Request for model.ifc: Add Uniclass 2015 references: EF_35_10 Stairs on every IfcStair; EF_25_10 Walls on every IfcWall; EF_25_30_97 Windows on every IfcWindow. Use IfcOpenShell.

First a look at what the model holds.

```python
import ifcopenshell

model = ifcopenshell.open("model.ifc")
print(model.schema)
print("classifications:", [c.Name for c in model.by_type("IfcClassification")])
for ifc_class in ("IfcDoor", "IfcRoof", "IfcStair", "IfcWall", "IfcWindow"):
    print(ifc_class, len(model.by_type(ifc_class)))
```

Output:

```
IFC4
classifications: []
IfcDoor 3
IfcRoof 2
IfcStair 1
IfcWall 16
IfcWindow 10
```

```python
import ifcopenshell
import ifcopenshell.api.classification

model = ifcopenshell.open("model.ifc")

system = ifcopenshell.api.classification.add_classification(model, classification="Uniclass 2015")

codes = {
    "IfcStair": ("EF_35_10", "Stairs"),
    "IfcWall": ("EF_25_10", "Walls"),
    "IfcWindow": ("EF_25_30_97", "Windows"),
}
for ifc_class, (code, name) in codes.items():
    products = model.by_type(ifc_class)
    ifcopenshell.api.classification.add_reference(
        model, products=products, classification=system, identification=code, name=name
    )
    print(code, len(products))

model.write("model_v2.ifc")
```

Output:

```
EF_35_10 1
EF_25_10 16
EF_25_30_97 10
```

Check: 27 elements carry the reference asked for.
